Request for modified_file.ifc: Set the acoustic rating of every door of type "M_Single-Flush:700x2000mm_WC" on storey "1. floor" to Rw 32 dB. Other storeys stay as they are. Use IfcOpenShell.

First a look at what the model holds.

```python
import ifcopenshell
import ifcopenshell.util.element

model = ifcopenshell.open("modified_file.ifc")
print(model.schema)
storey = next(s for s in model.by_type("IfcBuildingStorey") if s.Name == "1. floor")
doors = [e for e in ifcopenshell.util.element.get_decomposition(storey) if e.is_a("IfcDoor")]
seen = {}
for e in doors:
    element_type = ifcopenshell.util.element.get_type(e)
    key = (element_type.Name if element_type != e and element_type else None, ifcopenshell.util.element.get_pset(e, "Pset_DoorCommon", "AcousticRating"))
    seen[key] = seen.get(key, 0) + 1
for (name, value), count in sorted(seen.items(), key=str):
    print(count, "x", name, "|", value)
```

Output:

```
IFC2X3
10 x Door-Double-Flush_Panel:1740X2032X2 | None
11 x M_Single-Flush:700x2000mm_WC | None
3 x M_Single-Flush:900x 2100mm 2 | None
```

```python
import ifcopenshell
import ifcopenshell.api.pset
import ifcopenshell.util.element

model = ifcopenshell.open("modified_file.ifc")

storey = next(s for s in model.by_type("IfcBuildingStorey") if s.Name == "1. floor")
doors = [e for e in ifcopenshell.util.element.get_decomposition(storey) if e.is_a("IfcDoor")]

count = 0
for e in doors:
    element_type = ifcopenshell.util.element.get_type(e)
    if element_type in (None, e) or element_type.Name != "M_Single-Flush:700x2000mm_WC":
        continue
    # add_pset returns the element's existing set when there is one.
    pset = ifcopenshell.api.pset.add_pset(model, product=e, name="Pset_DoorCommon")
    ifcopenshell.api.pset.edit_pset(model, pset=pset, properties={"AcousticRating": "Rw 32 dB"})
    count += 1

print(count, "doors updated")

model.write("modified_file_updated.ifc")
```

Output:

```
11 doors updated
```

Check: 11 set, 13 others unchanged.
